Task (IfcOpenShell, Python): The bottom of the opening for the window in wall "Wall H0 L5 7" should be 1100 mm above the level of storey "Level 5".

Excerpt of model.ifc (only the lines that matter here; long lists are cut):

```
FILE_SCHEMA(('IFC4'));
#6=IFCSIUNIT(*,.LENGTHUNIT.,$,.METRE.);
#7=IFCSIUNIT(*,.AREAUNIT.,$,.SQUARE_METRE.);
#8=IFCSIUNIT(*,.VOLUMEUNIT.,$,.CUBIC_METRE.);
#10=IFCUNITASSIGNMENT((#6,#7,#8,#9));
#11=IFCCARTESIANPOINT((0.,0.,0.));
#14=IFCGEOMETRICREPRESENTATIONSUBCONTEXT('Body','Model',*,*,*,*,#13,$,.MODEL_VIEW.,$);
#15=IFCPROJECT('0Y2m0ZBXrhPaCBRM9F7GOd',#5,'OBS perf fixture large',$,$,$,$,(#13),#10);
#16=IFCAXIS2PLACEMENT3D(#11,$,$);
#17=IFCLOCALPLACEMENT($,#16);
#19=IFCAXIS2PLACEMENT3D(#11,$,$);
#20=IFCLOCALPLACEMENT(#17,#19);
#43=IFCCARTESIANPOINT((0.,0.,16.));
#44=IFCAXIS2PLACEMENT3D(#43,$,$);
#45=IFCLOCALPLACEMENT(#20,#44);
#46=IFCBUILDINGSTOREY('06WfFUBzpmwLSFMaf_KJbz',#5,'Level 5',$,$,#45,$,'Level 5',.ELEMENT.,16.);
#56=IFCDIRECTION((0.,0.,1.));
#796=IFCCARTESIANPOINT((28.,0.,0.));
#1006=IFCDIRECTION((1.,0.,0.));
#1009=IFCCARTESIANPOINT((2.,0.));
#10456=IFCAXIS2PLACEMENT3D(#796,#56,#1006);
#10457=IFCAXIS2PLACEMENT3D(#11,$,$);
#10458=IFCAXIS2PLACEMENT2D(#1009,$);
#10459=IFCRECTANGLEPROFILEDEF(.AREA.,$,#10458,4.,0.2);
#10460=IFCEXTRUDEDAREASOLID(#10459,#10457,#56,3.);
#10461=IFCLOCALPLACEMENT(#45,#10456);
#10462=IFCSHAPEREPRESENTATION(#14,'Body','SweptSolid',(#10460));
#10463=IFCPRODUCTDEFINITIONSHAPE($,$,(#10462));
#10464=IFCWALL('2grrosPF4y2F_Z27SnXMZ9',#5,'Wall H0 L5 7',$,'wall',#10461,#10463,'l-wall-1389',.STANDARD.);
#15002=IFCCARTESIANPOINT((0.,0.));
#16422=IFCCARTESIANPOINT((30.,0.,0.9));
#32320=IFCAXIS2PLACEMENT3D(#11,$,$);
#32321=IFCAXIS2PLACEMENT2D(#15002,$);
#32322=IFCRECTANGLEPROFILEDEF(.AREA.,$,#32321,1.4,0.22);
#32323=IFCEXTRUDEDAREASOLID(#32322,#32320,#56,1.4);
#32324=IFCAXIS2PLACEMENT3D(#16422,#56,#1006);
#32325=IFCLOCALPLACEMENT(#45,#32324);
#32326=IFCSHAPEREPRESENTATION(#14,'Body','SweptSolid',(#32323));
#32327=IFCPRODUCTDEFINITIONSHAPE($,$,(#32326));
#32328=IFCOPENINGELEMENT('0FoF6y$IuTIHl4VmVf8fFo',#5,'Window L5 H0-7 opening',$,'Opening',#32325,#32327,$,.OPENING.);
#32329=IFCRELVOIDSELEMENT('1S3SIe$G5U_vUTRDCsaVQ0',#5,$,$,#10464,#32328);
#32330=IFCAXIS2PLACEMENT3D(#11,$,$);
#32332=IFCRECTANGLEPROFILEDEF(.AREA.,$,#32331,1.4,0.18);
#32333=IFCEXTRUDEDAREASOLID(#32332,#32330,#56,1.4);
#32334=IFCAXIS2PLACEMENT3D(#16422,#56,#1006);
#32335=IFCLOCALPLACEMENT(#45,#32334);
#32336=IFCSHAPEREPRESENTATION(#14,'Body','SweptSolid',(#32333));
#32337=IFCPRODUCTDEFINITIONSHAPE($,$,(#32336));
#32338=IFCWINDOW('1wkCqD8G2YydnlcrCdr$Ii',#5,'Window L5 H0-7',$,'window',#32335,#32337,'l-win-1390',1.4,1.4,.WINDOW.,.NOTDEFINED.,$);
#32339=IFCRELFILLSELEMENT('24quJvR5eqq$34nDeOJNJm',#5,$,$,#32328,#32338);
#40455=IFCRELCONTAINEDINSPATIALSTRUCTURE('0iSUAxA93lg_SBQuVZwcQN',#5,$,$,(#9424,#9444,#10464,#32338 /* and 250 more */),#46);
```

```python
import numpy as np
import ifcopenshell
import ifcopenshell.api.geometry
import ifcopenshell.geom
import ifcopenshell.util.element
import ifcopenshell.util.placement
import ifcopenshell.util.shape
import ifcopenshell.util.unit

model = ifcopenshell.open("model.ifc")
unit_scale = ifcopenshell.util.unit.calculate_unit_scale(model)

window = model.by_guid("1wkCqD8G2YydnlcrCdr$Ii")
opening = window.FillsVoids[0].RelatingOpeningElement
storey = ifcopenshell.util.element.get_container(window, ifc_class="IfcBuildingStorey")
level = ifcopenshell.util.placement.get_local_placement(storey.ObjectPlacement)[2, 3]

# The opening's origin need not be at the sill, so measure its lowest point.
shape = ifcopenshell.geom.create_shape(ifcopenshell.geom.settings(), opening)
bottom = ifcopenshell.util.shape.get_shape_bottom_elevation(shape, shape.geometry) / unit_scale
dz = level + 1.1 - bottom

shift = np.array([0.0, 0.0, dz])
# The window is not placed relative to its opening, so move both.
for product in (opening, window):
    matrix = ifcopenshell.util.placement.get_local_placement(product.ObjectPlacement)
    matrix[:3, 3] += shift
    ifcopenshell.api.geometry.edit_object_placement(model, product=product, matrix=matrix, is_si=False)

print(f"moved by {dz * unit_scale:+.3f} m")

model.write("model_updated.ifc")
```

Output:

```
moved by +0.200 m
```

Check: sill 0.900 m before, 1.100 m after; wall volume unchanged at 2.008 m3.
